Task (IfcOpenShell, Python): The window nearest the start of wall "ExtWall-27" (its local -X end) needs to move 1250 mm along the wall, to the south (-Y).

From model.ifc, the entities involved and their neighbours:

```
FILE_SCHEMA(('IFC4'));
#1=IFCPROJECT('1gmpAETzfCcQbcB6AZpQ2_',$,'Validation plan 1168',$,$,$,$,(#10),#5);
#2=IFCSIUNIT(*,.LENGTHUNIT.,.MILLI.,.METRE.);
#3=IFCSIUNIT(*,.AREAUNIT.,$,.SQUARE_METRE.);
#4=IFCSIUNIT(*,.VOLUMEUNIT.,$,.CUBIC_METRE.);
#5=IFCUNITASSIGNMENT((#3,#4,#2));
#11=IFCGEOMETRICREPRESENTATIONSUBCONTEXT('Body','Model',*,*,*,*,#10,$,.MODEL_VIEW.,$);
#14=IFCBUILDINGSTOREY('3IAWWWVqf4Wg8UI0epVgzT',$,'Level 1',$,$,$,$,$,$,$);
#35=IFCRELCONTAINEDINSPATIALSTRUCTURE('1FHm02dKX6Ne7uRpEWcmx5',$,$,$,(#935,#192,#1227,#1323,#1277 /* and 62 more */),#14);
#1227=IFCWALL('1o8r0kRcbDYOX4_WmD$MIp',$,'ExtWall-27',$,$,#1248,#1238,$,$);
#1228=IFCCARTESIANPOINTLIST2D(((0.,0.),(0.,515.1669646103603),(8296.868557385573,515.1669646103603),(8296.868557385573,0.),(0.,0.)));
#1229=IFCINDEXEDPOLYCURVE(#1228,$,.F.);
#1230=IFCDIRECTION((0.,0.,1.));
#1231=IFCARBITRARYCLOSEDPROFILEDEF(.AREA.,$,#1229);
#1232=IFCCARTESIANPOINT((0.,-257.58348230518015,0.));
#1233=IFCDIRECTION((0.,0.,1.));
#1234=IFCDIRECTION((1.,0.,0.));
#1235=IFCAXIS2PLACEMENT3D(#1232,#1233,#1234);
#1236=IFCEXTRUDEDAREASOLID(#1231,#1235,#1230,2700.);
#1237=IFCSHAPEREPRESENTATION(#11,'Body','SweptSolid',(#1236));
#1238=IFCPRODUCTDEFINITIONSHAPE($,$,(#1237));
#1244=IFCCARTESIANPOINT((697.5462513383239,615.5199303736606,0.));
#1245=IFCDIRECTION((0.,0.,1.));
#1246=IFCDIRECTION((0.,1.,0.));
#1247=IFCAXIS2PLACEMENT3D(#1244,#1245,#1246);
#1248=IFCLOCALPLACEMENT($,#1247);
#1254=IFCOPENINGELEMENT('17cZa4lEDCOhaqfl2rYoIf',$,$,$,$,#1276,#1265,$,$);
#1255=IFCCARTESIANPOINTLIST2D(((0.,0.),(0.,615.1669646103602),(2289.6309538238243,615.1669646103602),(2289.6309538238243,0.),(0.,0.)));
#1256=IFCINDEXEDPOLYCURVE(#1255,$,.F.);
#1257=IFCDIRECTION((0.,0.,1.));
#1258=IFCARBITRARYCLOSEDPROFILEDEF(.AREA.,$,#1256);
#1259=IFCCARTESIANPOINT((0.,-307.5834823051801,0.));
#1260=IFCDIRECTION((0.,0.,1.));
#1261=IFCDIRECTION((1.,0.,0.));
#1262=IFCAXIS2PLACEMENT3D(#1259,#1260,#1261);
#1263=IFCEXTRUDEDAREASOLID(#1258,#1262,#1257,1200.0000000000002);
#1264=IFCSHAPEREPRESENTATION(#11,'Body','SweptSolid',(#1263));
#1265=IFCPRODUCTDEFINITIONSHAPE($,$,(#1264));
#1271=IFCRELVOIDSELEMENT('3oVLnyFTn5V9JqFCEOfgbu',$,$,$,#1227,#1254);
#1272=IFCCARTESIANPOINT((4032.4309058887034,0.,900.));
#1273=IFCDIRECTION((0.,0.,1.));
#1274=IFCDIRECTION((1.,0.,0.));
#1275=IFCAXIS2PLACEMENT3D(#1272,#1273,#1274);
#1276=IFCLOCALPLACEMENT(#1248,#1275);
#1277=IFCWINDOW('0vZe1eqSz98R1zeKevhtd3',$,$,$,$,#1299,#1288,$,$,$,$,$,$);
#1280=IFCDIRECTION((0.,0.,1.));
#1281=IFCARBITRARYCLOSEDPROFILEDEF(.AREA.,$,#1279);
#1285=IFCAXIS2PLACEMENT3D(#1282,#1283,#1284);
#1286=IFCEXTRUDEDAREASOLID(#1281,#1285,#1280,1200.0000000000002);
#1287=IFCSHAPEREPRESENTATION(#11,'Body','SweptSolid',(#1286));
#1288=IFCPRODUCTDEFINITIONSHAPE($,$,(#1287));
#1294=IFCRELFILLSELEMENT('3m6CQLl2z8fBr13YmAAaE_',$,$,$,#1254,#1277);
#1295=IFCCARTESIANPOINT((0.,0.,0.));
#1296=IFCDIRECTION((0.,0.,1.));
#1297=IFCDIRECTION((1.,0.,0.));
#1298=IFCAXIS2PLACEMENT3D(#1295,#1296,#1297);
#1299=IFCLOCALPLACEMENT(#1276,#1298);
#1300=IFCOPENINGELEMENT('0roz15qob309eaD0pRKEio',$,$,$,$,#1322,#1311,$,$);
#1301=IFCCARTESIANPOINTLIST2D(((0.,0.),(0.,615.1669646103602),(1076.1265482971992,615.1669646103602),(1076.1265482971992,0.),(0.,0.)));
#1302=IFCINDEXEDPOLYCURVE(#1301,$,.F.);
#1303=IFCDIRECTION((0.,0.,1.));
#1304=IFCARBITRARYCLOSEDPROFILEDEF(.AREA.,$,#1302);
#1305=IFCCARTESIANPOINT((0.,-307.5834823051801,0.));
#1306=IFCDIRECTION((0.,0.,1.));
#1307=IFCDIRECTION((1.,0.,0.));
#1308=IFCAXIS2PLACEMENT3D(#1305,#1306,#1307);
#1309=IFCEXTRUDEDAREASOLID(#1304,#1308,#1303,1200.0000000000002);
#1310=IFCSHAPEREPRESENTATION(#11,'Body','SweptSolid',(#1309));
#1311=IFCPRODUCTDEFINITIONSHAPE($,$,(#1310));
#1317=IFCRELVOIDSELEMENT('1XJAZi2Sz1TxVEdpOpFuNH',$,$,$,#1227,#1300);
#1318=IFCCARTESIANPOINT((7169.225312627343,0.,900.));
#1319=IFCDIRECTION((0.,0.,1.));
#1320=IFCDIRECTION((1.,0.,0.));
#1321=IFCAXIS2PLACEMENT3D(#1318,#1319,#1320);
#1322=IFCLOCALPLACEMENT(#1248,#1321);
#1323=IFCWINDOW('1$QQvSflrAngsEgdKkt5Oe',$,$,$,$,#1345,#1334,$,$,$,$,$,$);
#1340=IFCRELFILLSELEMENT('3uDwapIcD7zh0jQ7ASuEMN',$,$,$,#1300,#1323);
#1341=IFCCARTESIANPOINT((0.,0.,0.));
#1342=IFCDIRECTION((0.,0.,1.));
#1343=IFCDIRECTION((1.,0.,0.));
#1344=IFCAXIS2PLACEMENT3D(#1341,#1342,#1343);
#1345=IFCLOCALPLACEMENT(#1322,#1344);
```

```python
import ifcopenshell
import ifcopenshell.api.geometry
import ifcopenshell.util.placement

model = ifcopenshell.open("model.ifc")

window = model.by_id(1277)
opening = window.FillsVoids[0].RelatingOpeningElement
wall = opening.VoidsElements[0].RelatingBuildingElement

wall_matrix = ifcopenshell.util.placement.get_local_placement(wall.ObjectPlacement)
shift = wall_matrix[:3, 0] * -1250.0
before = ifcopenshell.util.placement.get_local_placement(window.ObjectPlacement)[:3, 3].copy()

# The window is placed relative to its opening, so it follows when the opening moves.
matrix = ifcopenshell.util.placement.get_local_placement(opening.ObjectPlacement)
matrix[:3, 3] += shift
ifcopenshell.api.geometry.edit_object_placement(
    model, product=opening, matrix=matrix, is_si=False, should_transform_children=True
)

after = ifcopenshell.util.placement.get_local_placement(window.ObjectPlacement)[:3, 3]
print("window moved by", (after - before).round(3) + 0.0)

model.write("model_edited.ifc")
```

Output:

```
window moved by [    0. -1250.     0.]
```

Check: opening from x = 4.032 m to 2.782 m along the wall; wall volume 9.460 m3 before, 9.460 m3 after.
